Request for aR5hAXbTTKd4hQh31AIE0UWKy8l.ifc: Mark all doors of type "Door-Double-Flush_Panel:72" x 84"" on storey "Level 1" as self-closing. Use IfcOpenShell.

First a look at what the model holds.

```python
import ifcopenshell
import ifcopenshell.util.element

model = ifcopenshell.open("aR5hAXbTTKd4hQh31AIE0UWKy8l.ifc")
print(model.schema)
storey = next(s for s in model.by_type("IfcBuildingStorey") if s.Name == "Level 1")
doors = [e for e in ifcopenshell.util.element.get_decomposition(storey) if e.is_a("IfcDoor")]
seen = {}
for e in doors:
    element_type = ifcopenshell.util.element.get_type(e)
    key = (element_type.Name if element_type != e and element_type else None, ifcopenshell.util.element.get_pset(e, "Pset_DoorCommon", "SelfClosing"))
    seen[key] = seen.get(key, 0) + 1
for (name, value), count in sorted(seen.items(), key=str):
    print(count, "x", name, "|", value)
```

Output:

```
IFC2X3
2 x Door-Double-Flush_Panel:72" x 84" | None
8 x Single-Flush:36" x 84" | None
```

```python
import ifcopenshell
import ifcopenshell.api.pset
import ifcopenshell.util.element

model = ifcopenshell.open("aR5hAXbTTKd4hQh31AIE0UWKy8l.ifc")

storey = next(s for s in model.by_type("IfcBuildingStorey") if s.Name == "Level 1")
doors = [e for e in ifcopenshell.util.element.get_decomposition(storey) if e.is_a("IfcDoor")]

count = 0
for e in doors:
    element_type = ifcopenshell.util.element.get_type(e)
    if element_type in (None, e) or element_type.Name != 'Door-Double-Flush_Panel:72" x 84"':
        continue
    # add_pset returns the element's existing set when there is one.
    pset = ifcopenshell.api.pset.add_pset(model, product=e, name="Pset_DoorCommon")
    ifcopenshell.api.pset.edit_pset(model, pset=pset, properties={"SelfClosing": True})
    count += 1

print(count, "doors updated")

model.write("aR5hAXbTTKd4hQh31AIE0UWKy8l-out.ifc")
```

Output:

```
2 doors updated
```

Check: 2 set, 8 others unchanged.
